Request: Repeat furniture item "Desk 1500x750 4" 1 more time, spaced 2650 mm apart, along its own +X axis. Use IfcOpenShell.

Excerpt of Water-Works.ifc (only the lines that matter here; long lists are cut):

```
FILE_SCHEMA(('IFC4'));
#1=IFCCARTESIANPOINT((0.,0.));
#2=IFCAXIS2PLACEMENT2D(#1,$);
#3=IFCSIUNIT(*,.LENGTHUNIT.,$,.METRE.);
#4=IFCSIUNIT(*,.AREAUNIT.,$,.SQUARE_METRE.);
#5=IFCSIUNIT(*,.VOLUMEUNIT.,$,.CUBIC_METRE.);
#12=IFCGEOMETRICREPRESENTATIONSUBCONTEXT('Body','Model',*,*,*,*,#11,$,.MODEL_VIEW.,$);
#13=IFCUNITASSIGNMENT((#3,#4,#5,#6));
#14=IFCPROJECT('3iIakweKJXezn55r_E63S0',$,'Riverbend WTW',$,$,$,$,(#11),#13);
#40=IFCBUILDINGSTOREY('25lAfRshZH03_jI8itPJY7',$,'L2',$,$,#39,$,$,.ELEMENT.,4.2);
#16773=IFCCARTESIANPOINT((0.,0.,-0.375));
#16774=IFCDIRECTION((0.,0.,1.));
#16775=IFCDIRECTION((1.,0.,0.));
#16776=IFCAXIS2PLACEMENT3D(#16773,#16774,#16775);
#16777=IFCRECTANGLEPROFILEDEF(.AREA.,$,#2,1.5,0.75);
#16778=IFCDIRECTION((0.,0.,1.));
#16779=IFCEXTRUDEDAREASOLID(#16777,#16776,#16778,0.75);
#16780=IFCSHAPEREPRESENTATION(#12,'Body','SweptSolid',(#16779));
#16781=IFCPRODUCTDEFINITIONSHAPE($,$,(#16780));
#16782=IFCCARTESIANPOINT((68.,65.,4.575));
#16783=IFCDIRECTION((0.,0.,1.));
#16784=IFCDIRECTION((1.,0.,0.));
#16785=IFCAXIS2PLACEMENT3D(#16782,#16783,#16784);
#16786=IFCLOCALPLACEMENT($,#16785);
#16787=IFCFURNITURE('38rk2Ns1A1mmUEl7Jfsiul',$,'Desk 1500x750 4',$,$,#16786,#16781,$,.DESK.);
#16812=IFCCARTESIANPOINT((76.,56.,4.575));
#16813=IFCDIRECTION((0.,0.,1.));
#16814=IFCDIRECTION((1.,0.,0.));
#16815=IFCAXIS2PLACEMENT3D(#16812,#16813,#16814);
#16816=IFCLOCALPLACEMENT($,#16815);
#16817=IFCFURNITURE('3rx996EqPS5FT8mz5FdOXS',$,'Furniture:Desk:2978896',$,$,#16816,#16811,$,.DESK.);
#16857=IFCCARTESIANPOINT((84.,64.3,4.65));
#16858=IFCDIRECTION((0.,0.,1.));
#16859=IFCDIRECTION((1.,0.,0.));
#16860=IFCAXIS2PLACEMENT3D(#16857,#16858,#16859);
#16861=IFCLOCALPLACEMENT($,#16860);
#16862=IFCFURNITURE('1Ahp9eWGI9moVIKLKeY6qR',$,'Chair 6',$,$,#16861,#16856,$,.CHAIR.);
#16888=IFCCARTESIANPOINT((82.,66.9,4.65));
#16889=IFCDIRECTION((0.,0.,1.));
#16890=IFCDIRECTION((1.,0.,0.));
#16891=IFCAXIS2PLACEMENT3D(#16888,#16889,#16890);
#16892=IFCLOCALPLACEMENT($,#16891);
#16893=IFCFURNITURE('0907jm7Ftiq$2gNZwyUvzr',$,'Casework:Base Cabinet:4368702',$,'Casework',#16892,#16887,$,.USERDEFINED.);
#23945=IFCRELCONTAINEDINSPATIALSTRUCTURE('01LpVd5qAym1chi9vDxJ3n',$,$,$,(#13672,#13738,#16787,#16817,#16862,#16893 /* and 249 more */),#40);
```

```python
import ifcopenshell
import ifcopenshell.api.geometry
import ifcopenshell.api.root
import ifcopenshell.util.element
import ifcopenshell.util.placement
import ifcopenshell.util.unit

model = ifcopenshell.open("Water-Works.ifc")
unit_scale = ifcopenshell.util.unit.calculate_unit_scale(model)

source = model.by_guid("38rk2Ns1A1mmUEl7Jfsiul")
base = ifcopenshell.util.placement.get_local_placement(source.ObjectPlacement)
step = base[:3, 0] * 2.65 / unit_scale

for i in range(1, 2):
    copy = ifcopenshell.api.root.copy_class(model, product=source)
    copy.Representation = ifcopenshell.util.element.copy_deep(
        model, source.Representation, exclude=["IfcGeometricRepresentationContext", "IfcRepresentationMap"]
    )
    matrix = base.copy()
    matrix[:3, 3] += i * step
    print("added at", matrix[:3, 3].round(3) + 0.0)
    ifcopenshell.api.geometry.edit_object_placement(model, product=copy, matrix=matrix, is_si=False)

model.write("Water-Works_rev.ifc")
```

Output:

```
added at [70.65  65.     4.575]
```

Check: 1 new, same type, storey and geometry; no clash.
